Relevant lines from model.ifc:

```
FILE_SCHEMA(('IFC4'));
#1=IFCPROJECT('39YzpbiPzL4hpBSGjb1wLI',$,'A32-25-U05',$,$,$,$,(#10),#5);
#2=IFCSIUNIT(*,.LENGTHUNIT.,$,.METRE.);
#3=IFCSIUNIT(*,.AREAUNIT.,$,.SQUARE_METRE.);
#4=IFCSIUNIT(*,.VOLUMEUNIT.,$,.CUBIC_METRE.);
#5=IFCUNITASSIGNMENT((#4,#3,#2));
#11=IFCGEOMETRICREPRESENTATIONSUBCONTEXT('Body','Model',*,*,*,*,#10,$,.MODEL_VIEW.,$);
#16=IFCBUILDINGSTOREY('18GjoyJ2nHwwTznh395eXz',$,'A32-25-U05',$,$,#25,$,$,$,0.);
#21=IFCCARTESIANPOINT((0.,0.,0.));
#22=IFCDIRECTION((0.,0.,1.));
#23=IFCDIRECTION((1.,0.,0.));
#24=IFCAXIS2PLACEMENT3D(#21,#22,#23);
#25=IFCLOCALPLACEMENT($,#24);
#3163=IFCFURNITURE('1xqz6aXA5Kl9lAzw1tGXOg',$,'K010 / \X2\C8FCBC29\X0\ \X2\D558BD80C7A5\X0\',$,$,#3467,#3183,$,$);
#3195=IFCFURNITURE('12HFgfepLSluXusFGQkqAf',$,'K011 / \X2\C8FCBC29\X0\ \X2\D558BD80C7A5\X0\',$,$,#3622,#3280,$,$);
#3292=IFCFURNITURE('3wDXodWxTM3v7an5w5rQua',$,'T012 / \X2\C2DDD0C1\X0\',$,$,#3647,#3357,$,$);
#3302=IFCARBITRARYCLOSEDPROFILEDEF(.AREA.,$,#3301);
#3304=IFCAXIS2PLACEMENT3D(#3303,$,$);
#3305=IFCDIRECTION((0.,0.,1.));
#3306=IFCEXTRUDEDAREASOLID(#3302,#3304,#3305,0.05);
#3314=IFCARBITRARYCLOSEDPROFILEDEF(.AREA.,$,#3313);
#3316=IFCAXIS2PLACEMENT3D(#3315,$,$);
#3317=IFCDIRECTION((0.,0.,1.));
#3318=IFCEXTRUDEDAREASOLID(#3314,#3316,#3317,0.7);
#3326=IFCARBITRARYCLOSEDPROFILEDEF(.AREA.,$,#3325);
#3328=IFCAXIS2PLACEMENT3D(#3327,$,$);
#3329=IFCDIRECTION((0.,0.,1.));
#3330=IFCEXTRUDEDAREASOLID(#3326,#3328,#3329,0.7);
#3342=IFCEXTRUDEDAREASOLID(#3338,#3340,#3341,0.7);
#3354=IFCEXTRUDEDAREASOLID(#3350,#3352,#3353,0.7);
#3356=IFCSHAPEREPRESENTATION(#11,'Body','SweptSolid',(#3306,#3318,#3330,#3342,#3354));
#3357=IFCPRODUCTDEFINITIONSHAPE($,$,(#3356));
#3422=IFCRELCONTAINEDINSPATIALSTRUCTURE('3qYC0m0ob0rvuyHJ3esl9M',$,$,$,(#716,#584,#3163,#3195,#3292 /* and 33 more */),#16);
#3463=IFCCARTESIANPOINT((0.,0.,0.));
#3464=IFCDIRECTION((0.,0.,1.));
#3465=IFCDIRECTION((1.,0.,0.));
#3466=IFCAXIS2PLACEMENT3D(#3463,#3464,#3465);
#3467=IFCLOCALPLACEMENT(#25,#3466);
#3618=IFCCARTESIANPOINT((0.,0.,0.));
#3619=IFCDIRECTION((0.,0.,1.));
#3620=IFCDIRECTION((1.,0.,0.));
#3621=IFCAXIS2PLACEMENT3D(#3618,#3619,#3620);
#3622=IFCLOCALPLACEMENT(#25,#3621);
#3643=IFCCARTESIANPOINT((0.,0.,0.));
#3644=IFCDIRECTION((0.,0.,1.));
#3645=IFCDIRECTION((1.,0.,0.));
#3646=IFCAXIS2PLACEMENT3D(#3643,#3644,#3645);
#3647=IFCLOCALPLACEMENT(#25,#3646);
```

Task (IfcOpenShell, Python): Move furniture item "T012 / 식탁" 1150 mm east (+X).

```python
import ifcopenshell
import ifcopenshell.api.geometry
import ifcopenshell.util.placement

model = ifcopenshell.open("model.ifc")

item = model.by_guid("3wDXodWxTM3v7an5w5rQua")
matrix = ifcopenshell.util.placement.get_local_placement(item.ObjectPlacement)
matrix[0, 3] += 1.15
ifcopenshell.api.geometry.edit_object_placement(model, product=item, matrix=matrix, is_si=False)

print(ifcopenshell.util.placement.get_local_placement(item.ObjectPlacement).round(3) + 0.0)

model.write("model-out.ifc")
```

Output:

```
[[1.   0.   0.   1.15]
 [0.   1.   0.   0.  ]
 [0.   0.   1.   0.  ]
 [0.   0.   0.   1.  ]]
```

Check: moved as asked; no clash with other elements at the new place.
